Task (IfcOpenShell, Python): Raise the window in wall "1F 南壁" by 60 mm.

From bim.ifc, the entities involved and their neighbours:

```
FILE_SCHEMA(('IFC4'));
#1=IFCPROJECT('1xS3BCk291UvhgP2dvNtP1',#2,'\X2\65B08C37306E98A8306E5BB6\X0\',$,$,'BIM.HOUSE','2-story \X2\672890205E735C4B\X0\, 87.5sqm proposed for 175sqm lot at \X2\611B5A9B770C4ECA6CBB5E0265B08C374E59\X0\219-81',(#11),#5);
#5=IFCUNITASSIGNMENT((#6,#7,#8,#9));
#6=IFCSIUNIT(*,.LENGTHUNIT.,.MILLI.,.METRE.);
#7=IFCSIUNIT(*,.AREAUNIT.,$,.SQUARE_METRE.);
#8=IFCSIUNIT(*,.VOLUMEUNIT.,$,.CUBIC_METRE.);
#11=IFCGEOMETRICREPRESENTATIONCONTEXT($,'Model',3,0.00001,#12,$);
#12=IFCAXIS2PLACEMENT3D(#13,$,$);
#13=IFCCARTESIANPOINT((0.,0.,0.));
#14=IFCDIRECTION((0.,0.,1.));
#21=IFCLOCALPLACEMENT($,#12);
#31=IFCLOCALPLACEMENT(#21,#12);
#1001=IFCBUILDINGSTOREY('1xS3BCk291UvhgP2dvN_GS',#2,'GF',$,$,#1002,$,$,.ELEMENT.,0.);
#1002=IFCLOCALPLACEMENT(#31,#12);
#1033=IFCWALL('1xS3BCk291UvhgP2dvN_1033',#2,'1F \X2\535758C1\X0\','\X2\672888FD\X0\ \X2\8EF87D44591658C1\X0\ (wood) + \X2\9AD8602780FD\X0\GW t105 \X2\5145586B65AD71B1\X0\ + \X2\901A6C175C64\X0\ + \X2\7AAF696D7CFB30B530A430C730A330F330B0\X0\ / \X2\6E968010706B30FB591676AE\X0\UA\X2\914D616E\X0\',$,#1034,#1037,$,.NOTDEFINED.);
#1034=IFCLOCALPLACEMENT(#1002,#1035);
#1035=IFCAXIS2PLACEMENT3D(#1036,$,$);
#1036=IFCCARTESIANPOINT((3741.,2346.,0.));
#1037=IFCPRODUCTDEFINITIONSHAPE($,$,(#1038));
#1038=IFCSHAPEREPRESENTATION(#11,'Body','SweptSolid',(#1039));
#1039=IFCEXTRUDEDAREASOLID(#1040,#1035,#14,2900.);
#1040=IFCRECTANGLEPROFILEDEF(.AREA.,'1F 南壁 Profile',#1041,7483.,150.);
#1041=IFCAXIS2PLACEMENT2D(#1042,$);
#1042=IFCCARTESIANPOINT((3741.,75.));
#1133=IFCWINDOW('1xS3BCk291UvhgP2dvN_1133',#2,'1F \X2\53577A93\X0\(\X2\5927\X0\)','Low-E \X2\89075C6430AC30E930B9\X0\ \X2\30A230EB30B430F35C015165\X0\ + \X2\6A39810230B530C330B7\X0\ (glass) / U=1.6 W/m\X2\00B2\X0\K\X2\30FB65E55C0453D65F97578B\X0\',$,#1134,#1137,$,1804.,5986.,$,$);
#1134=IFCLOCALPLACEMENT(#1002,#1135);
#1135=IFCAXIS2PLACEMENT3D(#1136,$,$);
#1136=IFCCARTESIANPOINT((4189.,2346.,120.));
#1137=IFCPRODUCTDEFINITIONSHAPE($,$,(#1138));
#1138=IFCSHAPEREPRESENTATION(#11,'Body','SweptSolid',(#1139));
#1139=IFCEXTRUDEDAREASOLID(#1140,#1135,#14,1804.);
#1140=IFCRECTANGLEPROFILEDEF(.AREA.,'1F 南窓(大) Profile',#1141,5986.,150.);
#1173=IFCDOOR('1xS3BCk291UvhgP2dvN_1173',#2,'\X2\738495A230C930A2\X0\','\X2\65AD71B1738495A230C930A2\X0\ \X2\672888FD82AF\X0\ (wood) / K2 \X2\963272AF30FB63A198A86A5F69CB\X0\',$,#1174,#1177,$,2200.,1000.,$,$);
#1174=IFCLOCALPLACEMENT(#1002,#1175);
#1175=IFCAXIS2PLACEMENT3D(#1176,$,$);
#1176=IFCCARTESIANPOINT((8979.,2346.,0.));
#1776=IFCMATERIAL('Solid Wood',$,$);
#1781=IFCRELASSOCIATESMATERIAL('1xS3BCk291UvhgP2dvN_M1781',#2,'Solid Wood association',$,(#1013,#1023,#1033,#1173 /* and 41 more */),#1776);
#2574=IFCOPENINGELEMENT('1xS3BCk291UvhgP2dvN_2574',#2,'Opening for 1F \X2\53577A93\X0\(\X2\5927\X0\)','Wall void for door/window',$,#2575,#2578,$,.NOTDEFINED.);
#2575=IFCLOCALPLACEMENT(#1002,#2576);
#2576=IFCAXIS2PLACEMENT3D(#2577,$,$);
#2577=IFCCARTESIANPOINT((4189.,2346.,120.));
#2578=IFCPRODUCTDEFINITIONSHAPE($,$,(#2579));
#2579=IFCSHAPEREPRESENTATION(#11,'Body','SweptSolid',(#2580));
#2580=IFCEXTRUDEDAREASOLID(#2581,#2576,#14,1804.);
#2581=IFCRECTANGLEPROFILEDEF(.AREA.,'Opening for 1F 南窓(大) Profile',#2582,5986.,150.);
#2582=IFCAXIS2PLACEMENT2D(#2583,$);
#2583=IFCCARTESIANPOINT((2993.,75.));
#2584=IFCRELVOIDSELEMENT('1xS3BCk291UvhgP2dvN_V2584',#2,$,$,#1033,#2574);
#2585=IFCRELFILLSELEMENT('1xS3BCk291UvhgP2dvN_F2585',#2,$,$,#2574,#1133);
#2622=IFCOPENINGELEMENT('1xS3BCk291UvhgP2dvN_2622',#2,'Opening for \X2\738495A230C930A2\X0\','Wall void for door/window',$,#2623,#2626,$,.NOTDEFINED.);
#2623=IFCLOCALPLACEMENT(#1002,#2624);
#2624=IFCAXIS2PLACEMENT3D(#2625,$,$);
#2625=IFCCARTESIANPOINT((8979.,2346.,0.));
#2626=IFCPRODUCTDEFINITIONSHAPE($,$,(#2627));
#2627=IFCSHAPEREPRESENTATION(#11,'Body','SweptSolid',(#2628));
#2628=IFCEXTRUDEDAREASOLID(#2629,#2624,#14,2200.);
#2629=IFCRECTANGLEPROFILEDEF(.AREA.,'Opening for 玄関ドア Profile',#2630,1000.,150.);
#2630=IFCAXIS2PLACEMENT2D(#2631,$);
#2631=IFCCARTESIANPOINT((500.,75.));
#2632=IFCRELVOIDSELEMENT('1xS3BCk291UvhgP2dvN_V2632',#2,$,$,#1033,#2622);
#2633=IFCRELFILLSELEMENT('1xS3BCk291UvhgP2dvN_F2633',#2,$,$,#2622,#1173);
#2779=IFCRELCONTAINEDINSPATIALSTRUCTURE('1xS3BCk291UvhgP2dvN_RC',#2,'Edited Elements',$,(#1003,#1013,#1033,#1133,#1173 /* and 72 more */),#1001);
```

```python
import numpy as np
import ifcopenshell
import ifcopenshell.api.geometry
import ifcopenshell.util.placement
import ifcopenshell.util.unit

model = ifcopenshell.open("bim.ifc")
unit_scale = ifcopenshell.util.unit.calculate_unit_scale(model)

window = model.by_guid("1xS3BCk291UvhgP2dvN_1133")
opening = window.FillsVoids[0].RelatingOpeningElement
dz = 60.0

shift = np.array([0.0, 0.0, dz])
# The window is not placed relative to its opening, so move both.
for product in (opening, window):
    matrix = ifcopenshell.util.placement.get_local_placement(product.ObjectPlacement)
    matrix[:3, 3] += shift
    ifcopenshell.api.geometry.edit_object_placement(model, product=product, matrix=matrix, is_si=False)

print(f"moved by {dz * unit_scale:+.3f} m")

model.write("bim_v2.ifc")
```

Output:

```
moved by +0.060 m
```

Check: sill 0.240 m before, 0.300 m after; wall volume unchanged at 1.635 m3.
